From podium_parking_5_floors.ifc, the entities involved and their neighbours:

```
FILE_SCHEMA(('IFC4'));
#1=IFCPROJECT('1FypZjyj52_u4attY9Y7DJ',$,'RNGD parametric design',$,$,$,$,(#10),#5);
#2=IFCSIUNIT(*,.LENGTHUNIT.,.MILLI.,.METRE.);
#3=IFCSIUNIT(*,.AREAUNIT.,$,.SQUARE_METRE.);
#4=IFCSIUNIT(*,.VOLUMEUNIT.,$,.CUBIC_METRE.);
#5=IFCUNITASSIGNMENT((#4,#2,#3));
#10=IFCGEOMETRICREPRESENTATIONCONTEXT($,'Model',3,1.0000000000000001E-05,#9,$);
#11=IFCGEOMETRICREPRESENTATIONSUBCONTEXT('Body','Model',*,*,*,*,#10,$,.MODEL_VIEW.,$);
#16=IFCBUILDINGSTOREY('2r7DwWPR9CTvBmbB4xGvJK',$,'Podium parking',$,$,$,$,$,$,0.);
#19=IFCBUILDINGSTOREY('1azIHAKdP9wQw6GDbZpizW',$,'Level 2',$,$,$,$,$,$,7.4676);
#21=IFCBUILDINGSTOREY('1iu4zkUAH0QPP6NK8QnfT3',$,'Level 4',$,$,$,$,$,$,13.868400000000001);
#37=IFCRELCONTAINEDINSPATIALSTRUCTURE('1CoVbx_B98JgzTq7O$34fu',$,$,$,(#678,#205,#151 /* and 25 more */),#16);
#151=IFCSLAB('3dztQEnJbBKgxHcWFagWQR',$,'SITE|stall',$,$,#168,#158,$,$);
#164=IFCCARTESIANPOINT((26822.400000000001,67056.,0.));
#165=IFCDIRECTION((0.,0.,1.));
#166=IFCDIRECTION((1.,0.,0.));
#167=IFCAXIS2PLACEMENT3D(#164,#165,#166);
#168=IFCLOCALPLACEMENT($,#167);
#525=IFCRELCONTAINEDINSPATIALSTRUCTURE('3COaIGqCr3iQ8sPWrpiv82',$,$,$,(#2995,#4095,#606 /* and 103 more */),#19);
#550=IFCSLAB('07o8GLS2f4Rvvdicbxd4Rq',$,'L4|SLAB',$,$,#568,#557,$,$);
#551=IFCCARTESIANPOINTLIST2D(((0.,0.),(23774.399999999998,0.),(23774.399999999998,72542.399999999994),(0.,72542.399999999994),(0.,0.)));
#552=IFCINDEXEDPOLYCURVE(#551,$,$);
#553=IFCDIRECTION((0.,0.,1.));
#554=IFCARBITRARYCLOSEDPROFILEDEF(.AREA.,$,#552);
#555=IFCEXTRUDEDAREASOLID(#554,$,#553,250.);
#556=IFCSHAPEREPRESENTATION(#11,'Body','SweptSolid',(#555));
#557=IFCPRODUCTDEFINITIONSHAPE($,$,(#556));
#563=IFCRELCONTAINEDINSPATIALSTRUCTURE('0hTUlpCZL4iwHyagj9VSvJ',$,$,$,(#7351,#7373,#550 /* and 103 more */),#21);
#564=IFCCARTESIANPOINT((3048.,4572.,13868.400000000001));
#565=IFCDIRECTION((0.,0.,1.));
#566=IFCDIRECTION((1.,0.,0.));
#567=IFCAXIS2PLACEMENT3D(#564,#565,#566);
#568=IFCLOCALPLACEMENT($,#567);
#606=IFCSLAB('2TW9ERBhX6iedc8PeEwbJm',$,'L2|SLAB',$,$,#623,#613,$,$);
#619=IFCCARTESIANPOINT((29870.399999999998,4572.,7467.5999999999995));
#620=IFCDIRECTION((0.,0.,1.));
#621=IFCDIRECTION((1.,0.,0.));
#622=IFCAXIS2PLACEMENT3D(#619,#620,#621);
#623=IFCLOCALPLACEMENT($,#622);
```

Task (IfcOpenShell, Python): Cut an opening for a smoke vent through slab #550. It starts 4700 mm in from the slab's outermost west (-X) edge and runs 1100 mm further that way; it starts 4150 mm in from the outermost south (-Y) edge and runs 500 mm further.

```python
import numpy as np
import ifcopenshell
import ifcopenshell.api.feature
import ifcopenshell.api.geometry
import ifcopenshell.api.root
import ifcopenshell.geom
import ifcopenshell.util.placement
import ifcopenshell.util.representation
import ifcopenshell.util.shape
import ifcopenshell.util.unit

model = ifcopenshell.open("podium_parking_5_floors.ifc")
unit_scale = ifcopenshell.util.unit.calculate_unit_scale(model)
settings = ifcopenshell.geom.settings()


def volume(element):
    """Net volume in cubic metres, openings subtracted."""
    shape = ifcopenshell.geom.create_shape(settings, element)
    return ifcopenshell.util.shape.get_volume(shape.geometry)


slab = model.by_id(550)
before = volume(slab)

# Extent in the slab's own axes, in metres. The edges named are its -X and -Y sides.
slab_shape = ifcopenshell.geom.create_shape(settings, slab)
vertices = ifcopenshell.util.shape.get_vertices(slab_shape.geometry)
x_min, y_min, bottom = vertices.min(axis=0)
top = vertices[:, 2].max()

opening = ifcopenshell.api.root.create_entity(model, ifc_class="IfcOpeningElement", name="Smoke vent opening", predefined_type="OPENING")
context = ifcopenshell.util.representation.get_context(model, "Model", "Body", "MODEL_VIEW")
width, depth = 1.1, 0.5
outline = [(0.0, 0.0), (width, 0.0), (width, depth), (0.0, depth), (0.0, 0.0)]
# Overshoot both faces by 50 mm so the cut is clean.
shape = ifcopenshell.api.geometry.add_slab_representation(
    model, context=context, depth=top - bottom + 0.1, polyline=outline
)
ifcopenshell.api.geometry.assign_representation(model, product=opening, representation=shape)

matrix = ifcopenshell.util.placement.get_local_placement(slab.ObjectPlacement)
matrix[:, 3] = matrix @ np.append(np.array([x_min + 4.7, y_min + 4.15, bottom - 0.05]) / unit_scale, 1.0)
ifcopenshell.api.geometry.edit_object_placement(model, product=opening, matrix=matrix, is_si=False)
ifcopenshell.api.feature.add_feature(model, feature=opening, element=slab)

after = volume(slab)

print(f"slab volume {before:.3f} -> {after:.3f} m3")

model.write("podium_parking_5_floors_v2.ifc")
```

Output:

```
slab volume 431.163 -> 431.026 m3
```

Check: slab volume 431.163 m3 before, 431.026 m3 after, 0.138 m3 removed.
